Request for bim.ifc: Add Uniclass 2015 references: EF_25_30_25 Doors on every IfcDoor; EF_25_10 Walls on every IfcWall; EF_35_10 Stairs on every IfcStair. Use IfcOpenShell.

First a look at what the model holds.

```python
import ifcopenshell

model = ifcopenshell.open("bim.ifc")
print(model.schema)
print("classifications:", [c.Name for c in model.by_type("IfcClassification")])
for ifc_class in ("IfcDoor", "IfcRoof", "IfcStair", "IfcWall", "IfcWindow"):
    print(ifc_class, len(model.by_type(ifc_class)))
```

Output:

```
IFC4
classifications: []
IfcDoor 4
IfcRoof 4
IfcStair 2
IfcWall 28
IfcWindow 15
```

```python
import ifcopenshell
import ifcopenshell.api.classification

model = ifcopenshell.open("bim.ifc")

system = ifcopenshell.api.classification.add_classification(model, classification="Uniclass 2015")

codes = {
    "IfcDoor": ("EF_25_30_25", "Doors"),
    "IfcWall": ("EF_25_10", "Walls"),
    "IfcStair": ("EF_35_10", "Stairs"),
}
for ifc_class, (code, name) in codes.items():
    products = model.by_type(ifc_class)
    ifcopenshell.api.classification.add_reference(
        model, products=products, classification=system, identification=code, name=name
    )
    print(code, len(products))

model.write("bim-out.ifc")
```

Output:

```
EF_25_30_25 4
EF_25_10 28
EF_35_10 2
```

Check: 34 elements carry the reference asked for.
